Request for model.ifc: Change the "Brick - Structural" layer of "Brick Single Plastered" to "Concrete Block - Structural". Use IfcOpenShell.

First a look at what the model holds.

```python
import ifcopenshell
import ifcopenshell.util.element

model = ifcopenshell.open("model.ifc")
print(model.schema)
for layer_set in model.by_type("IfcMaterialLayerSet"):
    if layer_set.LayerSetName == "Brick Single Plastered":
        for layer in layer_set.MaterialLayers:
            print(layer.id(), layer.Material and layer.Material.Name, layer.LayerThickness, sep=" | ")
        print(len(ifcopenshell.util.element.get_elements_by_material(model, layer_set)), "elements and types use it")
print(sorted(m.Name for m in model.by_type("IfcMaterial") if m.Name)[:60])
```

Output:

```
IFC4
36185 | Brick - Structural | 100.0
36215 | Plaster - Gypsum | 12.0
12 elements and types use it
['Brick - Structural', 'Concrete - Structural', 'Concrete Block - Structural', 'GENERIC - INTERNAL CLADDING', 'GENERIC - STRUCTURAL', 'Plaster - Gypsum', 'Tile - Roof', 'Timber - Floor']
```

```python
import ifcopenshell
import ifcopenshell.api.material

model = ifcopenshell.open("model.ifc")

layer_set = next(s for s in model.by_type("IfcMaterialLayerSet") if s.LayerSetName == "Brick Single Plastered")
layer = next(l for l in layer_set.MaterialLayers if l.Material and l.Material.Name == "Brick - Structural")
material = next(m for m in model.by_type("IfcMaterial") if m.Name == "Concrete Block - Structural")

# Point this one layer at the other material; renaming the old one would change it everywhere.
ifcopenshell.api.material.edit_layer(model, layer=layer, attributes={}, material=material)

print([l.Material.Name if l.Material else None for l in layer_set.MaterialLayers])

model.write("model_updated.ifc")
```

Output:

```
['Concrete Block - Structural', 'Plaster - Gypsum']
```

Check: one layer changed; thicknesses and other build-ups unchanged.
